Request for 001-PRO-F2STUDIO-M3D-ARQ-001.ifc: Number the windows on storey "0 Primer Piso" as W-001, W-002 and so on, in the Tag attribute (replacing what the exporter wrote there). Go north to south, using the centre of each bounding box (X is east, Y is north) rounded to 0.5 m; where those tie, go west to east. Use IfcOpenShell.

First a look at what the model holds.

```python
import ifcopenshell
import ifcopenshell.util.element
import ifcopenshell.util.placement

model = ifcopenshell.open("001-PRO-F2STUDIO-M3D-ARQ-001.ifc")
print(model.schema)
storey = next(s for s in model.by_type("IfcBuildingStorey") if s.Name == "0 Primer Piso")
windows = [e for e in ifcopenshell.util.element.get_decomposition(storey) if e.is_a("IfcWindow")]
for e in sorted(windows, key=lambda e: e.id()):
    origin = ifcopenshell.util.placement.get_local_placement(e.ObjectPlacement)[:3, 3]
    print(e.id(), e.Tag, e.Name, origin.round(2) + 0.0, sep=" | ")
```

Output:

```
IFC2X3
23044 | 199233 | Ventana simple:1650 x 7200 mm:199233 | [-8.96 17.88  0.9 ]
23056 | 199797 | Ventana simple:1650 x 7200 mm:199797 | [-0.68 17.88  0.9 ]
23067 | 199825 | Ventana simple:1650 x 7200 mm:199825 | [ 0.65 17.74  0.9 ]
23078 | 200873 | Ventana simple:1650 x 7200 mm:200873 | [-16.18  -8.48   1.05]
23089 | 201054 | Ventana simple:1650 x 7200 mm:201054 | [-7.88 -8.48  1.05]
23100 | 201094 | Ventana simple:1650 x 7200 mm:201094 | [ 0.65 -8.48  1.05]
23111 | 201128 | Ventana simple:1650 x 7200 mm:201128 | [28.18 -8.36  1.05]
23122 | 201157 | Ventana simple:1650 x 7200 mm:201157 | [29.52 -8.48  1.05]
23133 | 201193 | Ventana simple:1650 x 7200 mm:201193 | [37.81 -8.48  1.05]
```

```python
import ifcopenshell
import ifcopenshell.geom
import ifcopenshell.util.element
import ifcopenshell.util.shape

model = ifcopenshell.open("001-PRO-F2STUDIO-M3D-ARQ-001.ifc")
settings = ifcopenshell.geom.settings()
settings.set("use-world-coords", True)


def centre(element):
    shape = ifcopenshell.geom.create_shape(settings, element)
    return ifcopenshell.util.shape.get_bbox_centroid(shape.geometry)


storey = next(s for s in model.by_type("IfcBuildingStorey") if s.Name == "0 Primer Piso")
windows = [e for e in ifcopenshell.util.element.get_decomposition(storey) if e.is_a("IfcWindow")]

# Insertion points can sit at a corner or the storey origin, so sort by the geometry (in metres).
centres = {e: centre(e) for e in windows}
windows.sort(key=lambda e: (-round(centres[e][1] / 0.5), centres[e][0]))

for i, e in enumerate(windows, start=1):
    number = f"W-0{i:02d}"
    e.Tag = number
    print(e.id(), number)

model.write("001-PRO-F2STUDIO-M3D-ARQ-001_edited.ifc")
```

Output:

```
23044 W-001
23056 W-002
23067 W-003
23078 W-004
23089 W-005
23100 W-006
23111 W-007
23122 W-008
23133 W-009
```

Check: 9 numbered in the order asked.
